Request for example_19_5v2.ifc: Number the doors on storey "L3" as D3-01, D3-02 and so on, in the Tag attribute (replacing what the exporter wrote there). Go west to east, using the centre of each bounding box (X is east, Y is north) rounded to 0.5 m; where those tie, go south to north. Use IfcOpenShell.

First a look at what the model holds.

```python
import ifcopenshell
import ifcopenshell.util.element
import ifcopenshell.util.placement

model = ifcopenshell.open("example_19_5v2.ifc")
print(model.schema)
storey = next(s for s in model.by_type("IfcBuildingStorey") if s.Name == "L3")
doors = [e for e in ifcopenshell.util.element.get_decomposition(storey) if e.is_a("IfcDoor")]
for e in sorted(doors, key=lambda e: e.id()):
    origin = ifcopenshell.util.placement.get_local_placement(e.ObjectPlacement)[:3, 3]
    print(e.id(), e.Tag, e.Name, origin.round(2) + 0.0, sep=" | ")
```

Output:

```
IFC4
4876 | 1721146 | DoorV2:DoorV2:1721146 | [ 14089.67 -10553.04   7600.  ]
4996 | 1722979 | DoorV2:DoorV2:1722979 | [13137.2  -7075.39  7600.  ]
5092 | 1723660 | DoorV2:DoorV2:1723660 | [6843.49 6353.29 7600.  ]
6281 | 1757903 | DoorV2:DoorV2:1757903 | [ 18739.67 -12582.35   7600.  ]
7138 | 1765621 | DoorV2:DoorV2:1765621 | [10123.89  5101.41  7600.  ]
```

```python
import ifcopenshell
import ifcopenshell.geom
import ifcopenshell.util.element
import ifcopenshell.util.shape

model = ifcopenshell.open("example_19_5v2.ifc")
settings = ifcopenshell.geom.settings()
settings.set("use-world-coords", True)


def centre(element):
    shape = ifcopenshell.geom.create_shape(settings, element)
    return ifcopenshell.util.shape.get_bbox_centroid(shape.geometry)


storey = next(s for s in model.by_type("IfcBuildingStorey") if s.Name == "L3")
doors = [e for e in ifcopenshell.util.element.get_decomposition(storey) if e.is_a("IfcDoor")]

# Insertion points can sit at a corner or the storey origin, so sort by the geometry (in metres).
centres = {e: centre(e) for e in doors}
doors.sort(key=lambda e: (round(centres[e][0] / 0.5), centres[e][1]))

for i, e in enumerate(doors, start=1):
    number = f"D3-{i:02d}"
    e.Tag = number
    print(e.id(), number)

model.write("example_19_5v2_v2.ifc")
```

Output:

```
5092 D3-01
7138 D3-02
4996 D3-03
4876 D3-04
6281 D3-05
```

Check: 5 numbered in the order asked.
